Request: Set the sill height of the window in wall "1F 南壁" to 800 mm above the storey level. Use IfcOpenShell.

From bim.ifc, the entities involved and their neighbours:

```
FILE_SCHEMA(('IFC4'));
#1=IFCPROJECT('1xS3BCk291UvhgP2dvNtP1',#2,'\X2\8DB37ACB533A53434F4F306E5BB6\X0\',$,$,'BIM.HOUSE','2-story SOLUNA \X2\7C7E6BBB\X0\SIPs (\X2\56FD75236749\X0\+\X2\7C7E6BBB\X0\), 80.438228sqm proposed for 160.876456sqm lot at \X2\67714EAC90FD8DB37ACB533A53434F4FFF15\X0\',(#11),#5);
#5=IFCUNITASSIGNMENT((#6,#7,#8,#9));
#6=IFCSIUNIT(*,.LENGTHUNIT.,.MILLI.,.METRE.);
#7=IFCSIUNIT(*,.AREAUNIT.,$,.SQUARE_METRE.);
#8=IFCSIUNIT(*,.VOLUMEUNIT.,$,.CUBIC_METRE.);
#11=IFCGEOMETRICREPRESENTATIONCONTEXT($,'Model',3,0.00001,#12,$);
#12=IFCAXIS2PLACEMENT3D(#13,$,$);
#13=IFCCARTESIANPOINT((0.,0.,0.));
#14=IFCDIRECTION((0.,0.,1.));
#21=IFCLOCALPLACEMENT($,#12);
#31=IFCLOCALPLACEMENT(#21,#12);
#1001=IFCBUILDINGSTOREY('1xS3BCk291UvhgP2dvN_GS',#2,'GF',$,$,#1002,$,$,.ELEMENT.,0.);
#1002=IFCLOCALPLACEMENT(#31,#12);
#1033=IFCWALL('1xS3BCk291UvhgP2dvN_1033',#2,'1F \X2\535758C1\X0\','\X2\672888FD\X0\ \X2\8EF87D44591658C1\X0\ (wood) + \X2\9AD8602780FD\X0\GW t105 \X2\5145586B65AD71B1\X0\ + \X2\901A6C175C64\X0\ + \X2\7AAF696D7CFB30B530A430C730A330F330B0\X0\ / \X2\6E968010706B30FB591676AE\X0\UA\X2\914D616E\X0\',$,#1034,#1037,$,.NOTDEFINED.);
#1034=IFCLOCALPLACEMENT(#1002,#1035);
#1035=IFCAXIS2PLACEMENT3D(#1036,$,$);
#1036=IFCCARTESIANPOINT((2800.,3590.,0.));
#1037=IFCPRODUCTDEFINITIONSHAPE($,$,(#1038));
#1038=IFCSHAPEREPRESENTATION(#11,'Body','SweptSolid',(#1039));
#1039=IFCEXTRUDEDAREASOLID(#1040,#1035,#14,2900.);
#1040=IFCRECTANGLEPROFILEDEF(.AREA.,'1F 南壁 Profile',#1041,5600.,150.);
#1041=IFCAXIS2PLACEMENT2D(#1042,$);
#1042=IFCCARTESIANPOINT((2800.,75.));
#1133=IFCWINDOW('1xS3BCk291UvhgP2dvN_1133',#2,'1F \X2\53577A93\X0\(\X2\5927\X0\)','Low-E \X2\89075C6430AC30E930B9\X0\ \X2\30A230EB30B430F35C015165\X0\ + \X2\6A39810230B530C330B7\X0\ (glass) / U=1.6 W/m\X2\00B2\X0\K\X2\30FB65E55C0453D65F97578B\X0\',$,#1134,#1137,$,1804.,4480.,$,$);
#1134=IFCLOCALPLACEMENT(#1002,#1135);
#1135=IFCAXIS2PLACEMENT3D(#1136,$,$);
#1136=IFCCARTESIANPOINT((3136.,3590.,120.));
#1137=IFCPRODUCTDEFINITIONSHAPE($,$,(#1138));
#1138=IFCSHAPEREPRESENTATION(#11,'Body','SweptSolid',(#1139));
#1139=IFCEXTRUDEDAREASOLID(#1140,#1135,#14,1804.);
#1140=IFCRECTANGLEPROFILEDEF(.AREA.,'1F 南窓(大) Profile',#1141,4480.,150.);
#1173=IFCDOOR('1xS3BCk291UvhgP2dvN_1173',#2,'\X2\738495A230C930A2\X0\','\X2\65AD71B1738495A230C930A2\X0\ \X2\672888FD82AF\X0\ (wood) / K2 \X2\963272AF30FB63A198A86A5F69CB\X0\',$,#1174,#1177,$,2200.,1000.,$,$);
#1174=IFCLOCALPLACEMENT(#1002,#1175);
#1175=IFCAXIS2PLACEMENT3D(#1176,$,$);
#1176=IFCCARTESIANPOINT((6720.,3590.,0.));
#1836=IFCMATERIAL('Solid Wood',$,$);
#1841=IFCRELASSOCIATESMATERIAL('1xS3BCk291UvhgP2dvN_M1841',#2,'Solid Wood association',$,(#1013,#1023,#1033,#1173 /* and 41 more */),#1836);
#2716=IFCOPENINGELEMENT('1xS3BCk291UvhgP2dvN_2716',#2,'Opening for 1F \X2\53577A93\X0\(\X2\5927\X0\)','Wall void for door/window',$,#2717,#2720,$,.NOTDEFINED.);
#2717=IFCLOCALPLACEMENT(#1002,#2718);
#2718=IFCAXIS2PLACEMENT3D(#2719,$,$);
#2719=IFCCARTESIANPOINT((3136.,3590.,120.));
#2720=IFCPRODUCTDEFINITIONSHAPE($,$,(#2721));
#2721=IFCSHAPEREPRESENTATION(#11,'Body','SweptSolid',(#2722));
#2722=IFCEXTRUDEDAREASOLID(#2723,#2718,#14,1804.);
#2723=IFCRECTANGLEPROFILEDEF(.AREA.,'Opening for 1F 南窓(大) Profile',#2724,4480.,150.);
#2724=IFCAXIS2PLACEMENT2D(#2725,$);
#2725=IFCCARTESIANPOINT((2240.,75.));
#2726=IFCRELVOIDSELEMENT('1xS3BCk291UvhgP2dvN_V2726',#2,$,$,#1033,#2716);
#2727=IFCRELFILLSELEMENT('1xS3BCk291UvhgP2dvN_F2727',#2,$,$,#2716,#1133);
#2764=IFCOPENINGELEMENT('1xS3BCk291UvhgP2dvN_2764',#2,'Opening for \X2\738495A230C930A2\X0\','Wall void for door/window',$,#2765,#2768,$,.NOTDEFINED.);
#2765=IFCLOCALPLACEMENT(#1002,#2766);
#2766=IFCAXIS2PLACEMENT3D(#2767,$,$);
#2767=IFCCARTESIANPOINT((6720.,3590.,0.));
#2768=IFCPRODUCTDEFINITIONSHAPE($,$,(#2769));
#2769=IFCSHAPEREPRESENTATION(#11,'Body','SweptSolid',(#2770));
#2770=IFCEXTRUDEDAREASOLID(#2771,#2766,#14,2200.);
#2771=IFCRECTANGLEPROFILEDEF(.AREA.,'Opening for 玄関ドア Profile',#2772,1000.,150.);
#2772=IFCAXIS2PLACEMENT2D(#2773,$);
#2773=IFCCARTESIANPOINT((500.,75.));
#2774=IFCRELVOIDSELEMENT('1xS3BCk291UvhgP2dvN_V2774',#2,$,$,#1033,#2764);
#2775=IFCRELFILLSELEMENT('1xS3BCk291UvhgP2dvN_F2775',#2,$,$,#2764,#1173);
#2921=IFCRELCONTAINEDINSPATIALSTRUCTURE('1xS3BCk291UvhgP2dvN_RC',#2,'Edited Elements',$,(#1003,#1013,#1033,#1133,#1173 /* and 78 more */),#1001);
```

```python
import numpy as np
import ifcopenshell
import ifcopenshell.api.geometry
import ifcopenshell.geom
import ifcopenshell.util.element
import ifcopenshell.util.placement
import ifcopenshell.util.shape
import ifcopenshell.util.unit

model = ifcopenshell.open("bim.ifc")
unit_scale = ifcopenshell.util.unit.calculate_unit_scale(model)

window = model.by_guid("1xS3BCk291UvhgP2dvN_1133")
opening = window.FillsVoids[0].RelatingOpeningElement
storey = ifcopenshell.util.element.get_container(window, ifc_class="IfcBuildingStorey")
level = ifcopenshell.util.placement.get_local_placement(storey.ObjectPlacement)[2, 3]

# The opening's origin need not be at the sill, so measure its lowest point.
shape = ifcopenshell.geom.create_shape(ifcopenshell.geom.settings(), opening)
bottom = ifcopenshell.util.shape.get_shape_bottom_elevation(shape, shape.geometry) / unit_scale
dz = level + 0.8 / unit_scale - bottom

shift = np.array([0.0, 0.0, dz])
# The window is not placed relative to its opening, so move both.
for product in (opening, window):
    matrix = ifcopenshell.util.placement.get_local_placement(product.ObjectPlacement)
    matrix[:3, 3] += shift
    ifcopenshell.api.geometry.edit_object_placement(model, product=product, matrix=matrix, is_si=False)

print(f"moved by {dz * unit_scale:+.3f} m")

model.write("bim_v2.ifc")
```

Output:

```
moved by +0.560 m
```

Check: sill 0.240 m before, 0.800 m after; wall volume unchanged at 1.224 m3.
